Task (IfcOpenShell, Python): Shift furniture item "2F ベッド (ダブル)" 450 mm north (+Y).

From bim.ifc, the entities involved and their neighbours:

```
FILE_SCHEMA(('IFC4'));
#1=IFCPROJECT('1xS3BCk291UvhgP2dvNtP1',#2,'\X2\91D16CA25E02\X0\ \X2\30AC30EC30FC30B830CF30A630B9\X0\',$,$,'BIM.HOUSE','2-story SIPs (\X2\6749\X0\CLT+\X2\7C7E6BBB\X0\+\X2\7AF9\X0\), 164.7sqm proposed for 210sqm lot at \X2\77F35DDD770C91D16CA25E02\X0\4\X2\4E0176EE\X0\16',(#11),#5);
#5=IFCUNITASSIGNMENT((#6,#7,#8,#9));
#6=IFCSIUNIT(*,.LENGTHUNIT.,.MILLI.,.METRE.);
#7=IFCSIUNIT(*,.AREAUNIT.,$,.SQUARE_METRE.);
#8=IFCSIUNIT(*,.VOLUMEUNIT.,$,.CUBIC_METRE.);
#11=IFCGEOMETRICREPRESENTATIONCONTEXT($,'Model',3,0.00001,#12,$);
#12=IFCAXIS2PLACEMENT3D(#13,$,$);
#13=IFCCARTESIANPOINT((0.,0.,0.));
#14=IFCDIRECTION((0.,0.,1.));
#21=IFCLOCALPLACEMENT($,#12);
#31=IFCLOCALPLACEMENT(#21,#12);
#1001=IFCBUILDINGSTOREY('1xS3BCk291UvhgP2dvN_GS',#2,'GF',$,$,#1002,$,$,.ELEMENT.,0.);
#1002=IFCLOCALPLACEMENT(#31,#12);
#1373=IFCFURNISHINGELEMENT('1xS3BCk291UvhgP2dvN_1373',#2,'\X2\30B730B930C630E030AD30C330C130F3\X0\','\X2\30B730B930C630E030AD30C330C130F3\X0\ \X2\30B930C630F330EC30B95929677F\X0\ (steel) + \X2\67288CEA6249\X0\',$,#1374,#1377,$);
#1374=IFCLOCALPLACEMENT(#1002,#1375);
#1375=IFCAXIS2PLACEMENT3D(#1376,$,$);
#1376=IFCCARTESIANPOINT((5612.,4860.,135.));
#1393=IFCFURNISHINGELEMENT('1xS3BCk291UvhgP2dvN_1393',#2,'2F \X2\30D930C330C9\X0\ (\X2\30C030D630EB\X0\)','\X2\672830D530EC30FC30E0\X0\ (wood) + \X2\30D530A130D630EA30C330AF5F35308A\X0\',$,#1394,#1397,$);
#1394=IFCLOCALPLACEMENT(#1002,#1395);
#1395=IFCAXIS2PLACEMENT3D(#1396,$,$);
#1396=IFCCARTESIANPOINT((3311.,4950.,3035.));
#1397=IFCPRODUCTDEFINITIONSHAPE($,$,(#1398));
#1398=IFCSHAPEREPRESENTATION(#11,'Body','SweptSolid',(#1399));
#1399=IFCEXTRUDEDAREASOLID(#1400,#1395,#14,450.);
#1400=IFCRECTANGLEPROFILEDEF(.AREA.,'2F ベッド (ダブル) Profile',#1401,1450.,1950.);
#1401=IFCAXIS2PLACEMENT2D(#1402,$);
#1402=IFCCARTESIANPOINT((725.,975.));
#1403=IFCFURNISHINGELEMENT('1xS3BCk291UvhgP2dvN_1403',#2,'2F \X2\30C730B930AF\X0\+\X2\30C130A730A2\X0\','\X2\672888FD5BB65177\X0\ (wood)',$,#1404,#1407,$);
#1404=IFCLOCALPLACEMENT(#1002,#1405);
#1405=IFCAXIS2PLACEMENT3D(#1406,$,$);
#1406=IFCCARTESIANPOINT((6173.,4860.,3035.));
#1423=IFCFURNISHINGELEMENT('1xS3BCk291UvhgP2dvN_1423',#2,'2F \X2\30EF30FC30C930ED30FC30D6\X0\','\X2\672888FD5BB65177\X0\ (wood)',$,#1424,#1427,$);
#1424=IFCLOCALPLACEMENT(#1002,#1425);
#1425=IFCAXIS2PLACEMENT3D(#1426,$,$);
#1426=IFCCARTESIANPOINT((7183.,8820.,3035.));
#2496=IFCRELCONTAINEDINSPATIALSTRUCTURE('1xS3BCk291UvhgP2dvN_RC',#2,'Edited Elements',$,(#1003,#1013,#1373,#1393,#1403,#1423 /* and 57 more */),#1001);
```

```python
import ifcopenshell
import ifcopenshell.api.geometry
import ifcopenshell.util.placement

model = ifcopenshell.open("bim.ifc")

item = model.by_guid("1xS3BCk291UvhgP2dvN_1393")
matrix = ifcopenshell.util.placement.get_local_placement(item.ObjectPlacement)
matrix[1, 3] += 450.0
ifcopenshell.api.geometry.edit_object_placement(model, product=item, matrix=matrix, is_si=False)

print(ifcopenshell.util.placement.get_local_placement(item.ObjectPlacement).round(3) + 0.0)

model.write("bim_updated.ifc")
```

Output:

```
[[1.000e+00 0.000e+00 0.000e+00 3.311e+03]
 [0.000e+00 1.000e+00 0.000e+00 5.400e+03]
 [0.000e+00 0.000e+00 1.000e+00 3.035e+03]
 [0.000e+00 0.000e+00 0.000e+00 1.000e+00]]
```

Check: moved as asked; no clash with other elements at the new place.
